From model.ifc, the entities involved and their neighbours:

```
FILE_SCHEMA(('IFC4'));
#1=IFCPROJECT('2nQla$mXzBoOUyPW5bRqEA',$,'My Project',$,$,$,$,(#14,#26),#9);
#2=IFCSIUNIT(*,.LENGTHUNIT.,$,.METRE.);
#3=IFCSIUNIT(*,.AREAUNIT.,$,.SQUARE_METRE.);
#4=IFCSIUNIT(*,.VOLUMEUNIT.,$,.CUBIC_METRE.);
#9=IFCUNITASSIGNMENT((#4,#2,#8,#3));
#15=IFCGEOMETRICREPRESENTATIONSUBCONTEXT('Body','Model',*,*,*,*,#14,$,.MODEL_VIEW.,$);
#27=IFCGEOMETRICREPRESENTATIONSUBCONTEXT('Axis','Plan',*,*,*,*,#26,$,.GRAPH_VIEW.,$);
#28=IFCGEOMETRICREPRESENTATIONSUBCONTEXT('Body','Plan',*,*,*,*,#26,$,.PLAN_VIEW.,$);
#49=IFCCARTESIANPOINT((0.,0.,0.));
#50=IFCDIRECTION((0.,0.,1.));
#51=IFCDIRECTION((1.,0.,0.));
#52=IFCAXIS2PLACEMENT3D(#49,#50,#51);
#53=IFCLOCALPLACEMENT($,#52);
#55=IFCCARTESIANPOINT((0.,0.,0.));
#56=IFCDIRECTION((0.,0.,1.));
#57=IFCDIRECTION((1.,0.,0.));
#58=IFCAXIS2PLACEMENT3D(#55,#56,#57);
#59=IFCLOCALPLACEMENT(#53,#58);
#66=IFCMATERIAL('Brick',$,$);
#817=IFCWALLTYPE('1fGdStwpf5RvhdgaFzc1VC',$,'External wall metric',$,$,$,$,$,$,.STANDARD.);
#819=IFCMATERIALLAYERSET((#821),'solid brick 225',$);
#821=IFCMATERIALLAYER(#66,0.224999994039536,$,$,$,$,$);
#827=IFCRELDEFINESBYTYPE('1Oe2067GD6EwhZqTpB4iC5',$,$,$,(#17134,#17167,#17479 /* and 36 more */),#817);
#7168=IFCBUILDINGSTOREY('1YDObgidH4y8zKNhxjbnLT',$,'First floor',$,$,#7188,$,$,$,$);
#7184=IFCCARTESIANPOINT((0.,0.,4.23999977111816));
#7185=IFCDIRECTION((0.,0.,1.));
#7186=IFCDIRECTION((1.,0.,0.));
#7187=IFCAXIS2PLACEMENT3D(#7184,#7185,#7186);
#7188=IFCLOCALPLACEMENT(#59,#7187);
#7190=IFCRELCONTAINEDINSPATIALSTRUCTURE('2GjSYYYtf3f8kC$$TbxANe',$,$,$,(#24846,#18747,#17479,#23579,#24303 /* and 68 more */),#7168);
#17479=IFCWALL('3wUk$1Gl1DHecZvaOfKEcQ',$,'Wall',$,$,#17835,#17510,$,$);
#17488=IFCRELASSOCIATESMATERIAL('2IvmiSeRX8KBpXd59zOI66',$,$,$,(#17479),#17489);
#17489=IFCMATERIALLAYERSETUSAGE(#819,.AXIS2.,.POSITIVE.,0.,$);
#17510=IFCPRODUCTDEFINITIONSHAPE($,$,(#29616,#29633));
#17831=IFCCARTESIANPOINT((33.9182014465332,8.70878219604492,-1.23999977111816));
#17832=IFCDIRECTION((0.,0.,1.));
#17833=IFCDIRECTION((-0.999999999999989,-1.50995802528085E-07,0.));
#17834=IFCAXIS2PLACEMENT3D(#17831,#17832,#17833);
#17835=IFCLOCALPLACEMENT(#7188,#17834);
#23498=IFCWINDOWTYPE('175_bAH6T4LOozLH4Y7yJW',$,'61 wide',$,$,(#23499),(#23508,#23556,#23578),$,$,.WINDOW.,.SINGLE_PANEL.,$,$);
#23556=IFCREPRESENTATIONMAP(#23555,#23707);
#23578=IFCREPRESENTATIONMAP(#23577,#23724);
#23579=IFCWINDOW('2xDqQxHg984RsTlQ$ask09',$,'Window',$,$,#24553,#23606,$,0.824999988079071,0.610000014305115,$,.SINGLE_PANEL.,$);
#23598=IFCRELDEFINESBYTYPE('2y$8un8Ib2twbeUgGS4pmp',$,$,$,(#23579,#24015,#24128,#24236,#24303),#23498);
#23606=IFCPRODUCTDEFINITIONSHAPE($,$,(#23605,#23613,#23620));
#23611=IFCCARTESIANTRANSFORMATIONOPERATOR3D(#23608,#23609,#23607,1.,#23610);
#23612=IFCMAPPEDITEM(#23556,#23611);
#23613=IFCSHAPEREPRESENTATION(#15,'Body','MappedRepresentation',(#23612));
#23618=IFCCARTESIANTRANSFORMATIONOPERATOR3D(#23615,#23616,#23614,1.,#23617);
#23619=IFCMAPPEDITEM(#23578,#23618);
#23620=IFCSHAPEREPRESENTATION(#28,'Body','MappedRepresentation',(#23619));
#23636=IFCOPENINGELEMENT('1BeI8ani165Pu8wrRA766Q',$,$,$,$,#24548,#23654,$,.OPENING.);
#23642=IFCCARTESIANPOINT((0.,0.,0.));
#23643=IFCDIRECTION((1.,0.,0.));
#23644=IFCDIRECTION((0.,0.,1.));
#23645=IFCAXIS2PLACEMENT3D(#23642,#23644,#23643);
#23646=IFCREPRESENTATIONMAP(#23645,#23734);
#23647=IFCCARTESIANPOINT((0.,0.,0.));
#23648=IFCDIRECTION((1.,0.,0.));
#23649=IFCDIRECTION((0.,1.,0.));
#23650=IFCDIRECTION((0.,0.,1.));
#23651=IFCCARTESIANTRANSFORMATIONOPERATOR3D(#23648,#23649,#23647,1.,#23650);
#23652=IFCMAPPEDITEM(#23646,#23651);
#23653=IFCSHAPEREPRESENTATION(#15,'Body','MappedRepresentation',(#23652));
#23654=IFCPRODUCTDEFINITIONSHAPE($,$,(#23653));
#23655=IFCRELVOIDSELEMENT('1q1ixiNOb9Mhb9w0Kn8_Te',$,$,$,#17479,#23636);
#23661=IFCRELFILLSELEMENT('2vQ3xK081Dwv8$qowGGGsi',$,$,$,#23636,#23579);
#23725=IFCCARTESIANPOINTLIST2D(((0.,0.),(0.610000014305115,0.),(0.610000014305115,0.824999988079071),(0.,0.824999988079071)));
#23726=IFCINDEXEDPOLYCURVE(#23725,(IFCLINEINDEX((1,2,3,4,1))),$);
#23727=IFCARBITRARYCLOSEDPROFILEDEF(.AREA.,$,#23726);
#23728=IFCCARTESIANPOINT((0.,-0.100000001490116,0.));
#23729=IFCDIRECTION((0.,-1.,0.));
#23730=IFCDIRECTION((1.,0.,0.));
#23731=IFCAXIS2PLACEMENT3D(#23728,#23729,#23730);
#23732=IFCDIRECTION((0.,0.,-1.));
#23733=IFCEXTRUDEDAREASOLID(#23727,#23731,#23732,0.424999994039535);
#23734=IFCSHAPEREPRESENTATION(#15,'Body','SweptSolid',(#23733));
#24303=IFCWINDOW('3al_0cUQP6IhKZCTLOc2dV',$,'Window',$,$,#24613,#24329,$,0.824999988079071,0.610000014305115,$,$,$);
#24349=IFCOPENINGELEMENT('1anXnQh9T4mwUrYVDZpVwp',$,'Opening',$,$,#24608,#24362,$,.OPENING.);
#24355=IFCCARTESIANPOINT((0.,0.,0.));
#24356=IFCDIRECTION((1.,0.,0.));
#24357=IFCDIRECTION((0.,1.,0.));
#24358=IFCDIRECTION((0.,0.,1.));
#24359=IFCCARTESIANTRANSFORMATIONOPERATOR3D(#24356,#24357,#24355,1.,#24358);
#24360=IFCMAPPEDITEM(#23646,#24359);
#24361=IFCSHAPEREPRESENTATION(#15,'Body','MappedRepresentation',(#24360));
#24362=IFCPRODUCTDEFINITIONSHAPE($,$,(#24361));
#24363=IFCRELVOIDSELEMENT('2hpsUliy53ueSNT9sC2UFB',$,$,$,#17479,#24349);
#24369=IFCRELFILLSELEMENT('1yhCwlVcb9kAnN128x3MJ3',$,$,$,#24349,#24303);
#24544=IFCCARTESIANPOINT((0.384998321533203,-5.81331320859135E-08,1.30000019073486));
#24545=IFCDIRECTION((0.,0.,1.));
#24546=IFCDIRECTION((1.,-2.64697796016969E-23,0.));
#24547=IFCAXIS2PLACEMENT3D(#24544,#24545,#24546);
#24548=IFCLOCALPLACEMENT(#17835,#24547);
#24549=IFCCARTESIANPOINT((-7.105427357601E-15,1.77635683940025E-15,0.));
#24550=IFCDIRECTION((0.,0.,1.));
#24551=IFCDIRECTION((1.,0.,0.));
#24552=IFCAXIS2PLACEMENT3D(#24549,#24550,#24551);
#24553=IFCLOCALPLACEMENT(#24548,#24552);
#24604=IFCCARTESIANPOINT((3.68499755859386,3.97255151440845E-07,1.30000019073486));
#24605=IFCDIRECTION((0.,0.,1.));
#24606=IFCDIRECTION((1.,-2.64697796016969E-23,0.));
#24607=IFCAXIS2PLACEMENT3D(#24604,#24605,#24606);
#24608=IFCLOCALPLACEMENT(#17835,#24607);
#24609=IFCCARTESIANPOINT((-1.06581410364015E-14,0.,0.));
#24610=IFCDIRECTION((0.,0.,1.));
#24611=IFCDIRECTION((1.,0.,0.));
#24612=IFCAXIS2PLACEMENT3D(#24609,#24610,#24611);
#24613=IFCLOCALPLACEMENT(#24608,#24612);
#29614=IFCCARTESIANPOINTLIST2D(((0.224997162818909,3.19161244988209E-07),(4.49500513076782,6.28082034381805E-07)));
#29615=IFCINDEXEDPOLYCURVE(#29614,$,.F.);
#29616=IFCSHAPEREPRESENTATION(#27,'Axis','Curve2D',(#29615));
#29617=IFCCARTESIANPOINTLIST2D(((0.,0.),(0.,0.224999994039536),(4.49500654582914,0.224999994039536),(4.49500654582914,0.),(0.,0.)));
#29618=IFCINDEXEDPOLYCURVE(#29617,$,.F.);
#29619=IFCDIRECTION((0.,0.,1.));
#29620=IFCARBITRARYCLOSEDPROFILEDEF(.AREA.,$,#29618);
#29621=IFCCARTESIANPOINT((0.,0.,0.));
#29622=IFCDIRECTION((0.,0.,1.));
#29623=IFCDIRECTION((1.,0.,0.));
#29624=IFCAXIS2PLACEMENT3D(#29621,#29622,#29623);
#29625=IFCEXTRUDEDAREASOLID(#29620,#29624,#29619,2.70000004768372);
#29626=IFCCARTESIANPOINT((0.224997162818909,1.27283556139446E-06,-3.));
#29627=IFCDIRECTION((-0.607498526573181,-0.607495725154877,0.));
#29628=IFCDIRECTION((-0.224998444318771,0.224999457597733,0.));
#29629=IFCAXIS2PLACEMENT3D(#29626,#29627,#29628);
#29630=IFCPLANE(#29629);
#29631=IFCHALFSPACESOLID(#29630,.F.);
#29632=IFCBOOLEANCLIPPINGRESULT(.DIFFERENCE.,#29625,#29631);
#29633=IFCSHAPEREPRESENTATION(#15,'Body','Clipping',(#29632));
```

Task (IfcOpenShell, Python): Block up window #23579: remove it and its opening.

```python
import ifcopenshell
import ifcopenshell.api.feature
import ifcopenshell.api.root
import ifcopenshell.geom
import ifcopenshell.util.shape

model = ifcopenshell.open("model.ifc")
settings = ifcopenshell.geom.settings()


def volume(element):
    """Net volume in cubic metres, openings subtracted."""
    shape = ifcopenshell.geom.create_shape(settings, element)
    return ifcopenshell.util.shape.get_volume(shape.geometry)


window = model.by_guid("2xDqQxHg984RsTlQ$ask09")
opening = window.FillsVoids[0].RelatingOpeningElement
wall = opening.VoidsElements[0].RelatingBuildingElement
before = volume(wall)

ifcopenshell.api.root.remove_product(model, product=window)
ifcopenshell.api.feature.remove_feature(model, feature=opening)

after = volume(wall)

print(f"wall volume {before:.3f} -> {after:.3f} m3")

model.write("model-out.ifc")
```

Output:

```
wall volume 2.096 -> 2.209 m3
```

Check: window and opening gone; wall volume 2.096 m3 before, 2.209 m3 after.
